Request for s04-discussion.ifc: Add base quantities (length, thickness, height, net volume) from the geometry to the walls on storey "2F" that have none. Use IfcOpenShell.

First a look at what the model holds.

```python
import ifcopenshell
import ifcopenshell.util.element
import ifcopenshell.util.unit

model = ifcopenshell.open("s04-discussion.ifc")
print(model.schema)
for unit_type in ("LENGTHUNIT", "AREAUNIT", "VOLUMEUNIT"):
    print(unit_type, ifcopenshell.util.unit.calculate_unit_scale(model, unit_type))
storey = next(s for s in model.by_type("IfcBuildingStorey") if s.Name == "2F")
walls = [e for e in ifcopenshell.util.element.get_decomposition(storey) if e.is_a("IfcWall")]
for e in sorted(walls, key=lambda e: e.id()):
    print(e.id(), e.is_a(), e.Name, list(ifcopenshell.util.element.get_psets(e, qtos_only=True)), sep=" | ")
```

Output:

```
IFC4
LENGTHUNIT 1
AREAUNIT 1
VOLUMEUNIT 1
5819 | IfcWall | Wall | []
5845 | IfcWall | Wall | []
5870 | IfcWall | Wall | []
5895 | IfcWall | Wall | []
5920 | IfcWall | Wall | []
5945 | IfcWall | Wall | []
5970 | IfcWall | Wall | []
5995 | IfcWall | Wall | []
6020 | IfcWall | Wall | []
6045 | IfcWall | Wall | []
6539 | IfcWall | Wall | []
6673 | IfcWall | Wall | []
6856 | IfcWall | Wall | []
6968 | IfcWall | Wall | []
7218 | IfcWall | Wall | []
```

```python
import ifcopenshell
import ifcopenshell.api.pset
import ifcopenshell.geom
import ifcopenshell.util.element
import ifcopenshell.util.shape
import ifcopenshell.util.unit

model = ifcopenshell.open("s04-discussion.ifc")
unit_scale = ifcopenshell.util.unit.calculate_unit_scale(model)
volume_scale = ifcopenshell.util.unit.calculate_unit_scale(model, "VOLUMEUNIT")
settings = ifcopenshell.geom.settings()

storey = next(s for s in model.by_type("IfcBuildingStorey") if s.Name == "2F")
walls = [e for e in ifcopenshell.util.element.get_decomposition(storey) if e.is_a("IfcWall")]

for e in sorted(walls, key=lambda e: e.id()):
    if ifcopenshell.util.element.get_psets(e, qtos_only=True, should_inherit=False):
        continue
    # Geometry comes back in metres, in the element's own axes.
    shape = ifcopenshell.geom.create_shape(settings, e)
    values = {
        "Length": ifcopenshell.util.shape.get_x(shape.geometry) / unit_scale,
        "Width": ifcopenshell.util.shape.get_y(shape.geometry) / unit_scale,
        "Height": ifcopenshell.util.shape.get_z(shape.geometry) / unit_scale,
        "NetVolume": ifcopenshell.util.shape.get_volume(shape.geometry) / volume_scale,
    }
    qto = ifcopenshell.api.pset.add_qto(model, product=e, name="Qto_WallBaseQuantities")
    ifcopenshell.api.pset.edit_qto(model, qto=qto, properties=values)
    print(e.id(), {k: round(v, 3) for k, v in values.items()})

model.write("s04-discussion_rev.ifc")
```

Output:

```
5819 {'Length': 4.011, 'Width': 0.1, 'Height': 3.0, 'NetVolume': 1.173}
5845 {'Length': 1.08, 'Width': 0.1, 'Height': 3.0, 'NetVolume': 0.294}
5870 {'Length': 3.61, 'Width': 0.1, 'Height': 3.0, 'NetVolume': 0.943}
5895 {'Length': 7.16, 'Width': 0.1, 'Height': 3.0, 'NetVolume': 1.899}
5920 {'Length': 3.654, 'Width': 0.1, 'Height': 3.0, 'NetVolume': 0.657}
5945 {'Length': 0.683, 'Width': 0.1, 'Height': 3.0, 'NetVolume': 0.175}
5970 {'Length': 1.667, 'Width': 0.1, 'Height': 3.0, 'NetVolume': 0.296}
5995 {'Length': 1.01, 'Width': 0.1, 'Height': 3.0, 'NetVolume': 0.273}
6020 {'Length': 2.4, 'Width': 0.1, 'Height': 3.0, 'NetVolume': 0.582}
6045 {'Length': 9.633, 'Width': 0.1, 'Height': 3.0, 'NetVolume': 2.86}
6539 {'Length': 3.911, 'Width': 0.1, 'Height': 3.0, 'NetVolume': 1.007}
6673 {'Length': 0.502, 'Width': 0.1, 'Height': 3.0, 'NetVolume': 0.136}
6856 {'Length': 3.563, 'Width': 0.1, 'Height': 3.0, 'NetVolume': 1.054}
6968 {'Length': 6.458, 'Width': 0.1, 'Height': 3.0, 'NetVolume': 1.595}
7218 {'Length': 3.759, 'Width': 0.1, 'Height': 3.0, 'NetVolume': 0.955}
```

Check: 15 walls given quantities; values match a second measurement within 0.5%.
